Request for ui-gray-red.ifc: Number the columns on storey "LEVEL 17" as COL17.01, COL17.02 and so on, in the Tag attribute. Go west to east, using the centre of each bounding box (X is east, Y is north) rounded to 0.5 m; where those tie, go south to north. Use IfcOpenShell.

First a look at what the model holds.

```python
import ifcopenshell
import ifcopenshell.util.element
import ifcopenshell.util.placement

model = ifcopenshell.open("ui-gray-red.ifc")
print(model.schema)
storey = next(s for s in model.by_type("IfcBuildingStorey") if s.Name == "LEVEL 17")
columns = [e for e in ifcopenshell.util.element.get_decomposition(storey) if e.is_a("IfcColumn")]
for e in sorted(columns, key=lambda e: e.id()):
    origin = ifcopenshell.util.placement.get_local_placement(e.ObjectPlacement)[:3, 3]
    print(e.id(), e.Tag, e.Name, origin.round(2) + 0.0, sep=" | ")
```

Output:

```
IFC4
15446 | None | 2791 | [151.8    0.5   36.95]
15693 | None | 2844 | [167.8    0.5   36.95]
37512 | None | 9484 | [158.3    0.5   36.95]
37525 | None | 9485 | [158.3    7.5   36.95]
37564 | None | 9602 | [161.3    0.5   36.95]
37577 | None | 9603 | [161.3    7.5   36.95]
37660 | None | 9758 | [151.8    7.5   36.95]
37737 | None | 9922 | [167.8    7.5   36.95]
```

```python
import ifcopenshell
import ifcopenshell.geom
import ifcopenshell.util.element
import ifcopenshell.util.shape

model = ifcopenshell.open("ui-gray-red.ifc")
settings = ifcopenshell.geom.settings()
settings.set("use-world-coords", True)


def centre(element):
    shape = ifcopenshell.geom.create_shape(settings, element)
    return ifcopenshell.util.shape.get_bbox_centroid(shape.geometry)


storey = next(s for s in model.by_type("IfcBuildingStorey") if s.Name == "LEVEL 17")
columns = [e for e in ifcopenshell.util.element.get_decomposition(storey) if e.is_a("IfcColumn")]

# Insertion points can sit at a corner or the storey origin, so sort by the geometry (in metres).
centres = {e: centre(e) for e in columns}
columns.sort(key=lambda e: (round(centres[e][0] / 0.5), centres[e][1]))

for i, e in enumerate(columns, start=1):
    number = f"COL17.{i:02d}"
    e.Tag = number
    print(e.id(), number)

model.write("ui-gray-red_updated.ifc")
```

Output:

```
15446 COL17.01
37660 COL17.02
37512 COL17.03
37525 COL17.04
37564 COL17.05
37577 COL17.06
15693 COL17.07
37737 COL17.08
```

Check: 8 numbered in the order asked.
